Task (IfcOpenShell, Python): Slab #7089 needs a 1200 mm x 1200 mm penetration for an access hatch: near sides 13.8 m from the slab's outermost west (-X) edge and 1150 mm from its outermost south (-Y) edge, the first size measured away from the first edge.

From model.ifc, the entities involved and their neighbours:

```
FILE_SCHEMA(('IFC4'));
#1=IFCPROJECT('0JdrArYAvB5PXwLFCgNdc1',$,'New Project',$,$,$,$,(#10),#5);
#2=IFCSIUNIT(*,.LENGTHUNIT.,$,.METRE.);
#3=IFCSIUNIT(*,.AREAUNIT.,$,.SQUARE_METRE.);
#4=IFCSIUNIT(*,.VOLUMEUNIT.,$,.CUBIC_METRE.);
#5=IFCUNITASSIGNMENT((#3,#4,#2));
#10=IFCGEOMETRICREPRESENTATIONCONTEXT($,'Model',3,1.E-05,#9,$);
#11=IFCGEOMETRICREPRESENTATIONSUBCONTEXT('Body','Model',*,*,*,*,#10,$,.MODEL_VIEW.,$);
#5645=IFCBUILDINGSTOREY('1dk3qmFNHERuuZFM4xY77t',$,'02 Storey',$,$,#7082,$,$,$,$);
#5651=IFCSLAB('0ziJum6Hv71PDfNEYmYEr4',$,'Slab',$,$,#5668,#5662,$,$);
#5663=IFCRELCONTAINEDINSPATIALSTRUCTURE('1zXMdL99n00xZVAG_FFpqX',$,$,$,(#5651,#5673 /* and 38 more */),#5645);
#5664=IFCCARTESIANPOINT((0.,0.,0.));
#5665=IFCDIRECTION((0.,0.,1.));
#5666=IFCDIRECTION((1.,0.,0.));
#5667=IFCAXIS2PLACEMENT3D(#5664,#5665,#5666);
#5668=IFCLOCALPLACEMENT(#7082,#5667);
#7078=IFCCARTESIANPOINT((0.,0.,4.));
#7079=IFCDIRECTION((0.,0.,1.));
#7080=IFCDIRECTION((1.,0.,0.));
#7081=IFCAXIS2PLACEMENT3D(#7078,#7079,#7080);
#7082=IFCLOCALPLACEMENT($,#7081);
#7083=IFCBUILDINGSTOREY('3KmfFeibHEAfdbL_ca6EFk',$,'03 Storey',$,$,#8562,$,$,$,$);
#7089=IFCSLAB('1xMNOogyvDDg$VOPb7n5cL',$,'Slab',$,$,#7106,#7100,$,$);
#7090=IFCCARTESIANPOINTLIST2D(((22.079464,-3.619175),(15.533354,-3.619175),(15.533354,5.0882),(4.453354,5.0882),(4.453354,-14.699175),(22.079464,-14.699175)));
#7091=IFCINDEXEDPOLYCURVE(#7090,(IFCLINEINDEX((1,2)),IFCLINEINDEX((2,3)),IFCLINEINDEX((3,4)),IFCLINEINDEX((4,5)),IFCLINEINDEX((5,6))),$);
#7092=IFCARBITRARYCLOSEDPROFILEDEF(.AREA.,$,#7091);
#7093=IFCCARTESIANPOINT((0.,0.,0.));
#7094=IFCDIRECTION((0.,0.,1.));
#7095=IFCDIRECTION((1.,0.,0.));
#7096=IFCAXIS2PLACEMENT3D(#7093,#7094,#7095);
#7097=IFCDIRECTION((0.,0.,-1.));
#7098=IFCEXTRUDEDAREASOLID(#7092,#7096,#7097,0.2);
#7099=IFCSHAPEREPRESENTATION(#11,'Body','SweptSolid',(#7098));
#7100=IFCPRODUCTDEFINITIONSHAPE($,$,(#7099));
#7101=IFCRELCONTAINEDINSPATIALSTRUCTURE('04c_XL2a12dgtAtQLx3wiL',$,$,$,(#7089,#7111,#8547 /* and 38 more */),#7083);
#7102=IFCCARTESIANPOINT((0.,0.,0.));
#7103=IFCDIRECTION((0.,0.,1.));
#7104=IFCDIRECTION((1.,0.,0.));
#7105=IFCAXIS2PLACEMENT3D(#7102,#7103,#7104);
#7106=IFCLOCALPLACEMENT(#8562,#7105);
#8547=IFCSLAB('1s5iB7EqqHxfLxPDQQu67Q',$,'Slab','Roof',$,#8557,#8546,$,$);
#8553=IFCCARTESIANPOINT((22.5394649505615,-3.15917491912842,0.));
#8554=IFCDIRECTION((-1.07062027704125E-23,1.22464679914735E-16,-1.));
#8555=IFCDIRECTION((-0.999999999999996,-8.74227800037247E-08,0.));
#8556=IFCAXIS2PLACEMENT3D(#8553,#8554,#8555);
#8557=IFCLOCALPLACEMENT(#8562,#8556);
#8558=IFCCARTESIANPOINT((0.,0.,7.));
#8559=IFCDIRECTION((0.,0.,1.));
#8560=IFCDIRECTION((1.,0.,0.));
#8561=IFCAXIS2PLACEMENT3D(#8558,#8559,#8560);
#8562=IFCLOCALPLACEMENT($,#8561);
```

```python
import numpy as np
import ifcopenshell
import ifcopenshell.api.feature
import ifcopenshell.api.geometry
import ifcopenshell.api.root
import ifcopenshell.geom
import ifcopenshell.util.placement
import ifcopenshell.util.representation
import ifcopenshell.util.shape
import ifcopenshell.util.unit

model = ifcopenshell.open("model.ifc")
unit_scale = ifcopenshell.util.unit.calculate_unit_scale(model)
settings = ifcopenshell.geom.settings()


def volume(element):
    """Net volume in cubic metres, openings subtracted."""
    shape = ifcopenshell.geom.create_shape(settings, element)
    return ifcopenshell.util.shape.get_volume(shape.geometry)


slab = model.by_guid("1xMNOogyvDDg$VOPb7n5cL")
before = volume(slab)

# Extent in the slab's own axes, in metres. The edges named are its -X and -Y sides.
slab_shape = ifcopenshell.geom.create_shape(settings, slab)
vertices = ifcopenshell.util.shape.get_vertices(slab_shape.geometry)
x_min, y_min, bottom = vertices.min(axis=0)
top = vertices[:, 2].max()

opening = ifcopenshell.api.root.create_entity(model, ifc_class="IfcOpeningElement", name="Access hatch opening", predefined_type="OPENING")
context = ifcopenshell.util.representation.get_context(model, "Model", "Body", "MODEL_VIEW")
width, depth = 1.2, 1.2
outline = [(0.0, 0.0), (width, 0.0), (width, depth), (0.0, depth), (0.0, 0.0)]
# Overshoot both faces by 50 mm so the cut is clean.
shape = ifcopenshell.api.geometry.add_slab_representation(
    model, context=context, depth=top - bottom + 0.1, polyline=outline
)
ifcopenshell.api.geometry.assign_representation(model, product=opening, representation=shape)

matrix = ifcopenshell.util.placement.get_local_placement(slab.ObjectPlacement)
matrix[:, 3] = matrix @ np.append(np.array([x_min + 13.8, y_min + 1.15, bottom - 0.05]) / unit_scale, 1.0)
ifcopenshell.api.geometry.edit_object_placement(model, product=opening, matrix=matrix, is_si=False)
ifcopenshell.api.feature.add_feature(model, feature=opening, element=slab)

after = volume(slab)

print(f"slab volume {before:.3f} -> {after:.3f} m3")

model.write("model_edited.ifc")
```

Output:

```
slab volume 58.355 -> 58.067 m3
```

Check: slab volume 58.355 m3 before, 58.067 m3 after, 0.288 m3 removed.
